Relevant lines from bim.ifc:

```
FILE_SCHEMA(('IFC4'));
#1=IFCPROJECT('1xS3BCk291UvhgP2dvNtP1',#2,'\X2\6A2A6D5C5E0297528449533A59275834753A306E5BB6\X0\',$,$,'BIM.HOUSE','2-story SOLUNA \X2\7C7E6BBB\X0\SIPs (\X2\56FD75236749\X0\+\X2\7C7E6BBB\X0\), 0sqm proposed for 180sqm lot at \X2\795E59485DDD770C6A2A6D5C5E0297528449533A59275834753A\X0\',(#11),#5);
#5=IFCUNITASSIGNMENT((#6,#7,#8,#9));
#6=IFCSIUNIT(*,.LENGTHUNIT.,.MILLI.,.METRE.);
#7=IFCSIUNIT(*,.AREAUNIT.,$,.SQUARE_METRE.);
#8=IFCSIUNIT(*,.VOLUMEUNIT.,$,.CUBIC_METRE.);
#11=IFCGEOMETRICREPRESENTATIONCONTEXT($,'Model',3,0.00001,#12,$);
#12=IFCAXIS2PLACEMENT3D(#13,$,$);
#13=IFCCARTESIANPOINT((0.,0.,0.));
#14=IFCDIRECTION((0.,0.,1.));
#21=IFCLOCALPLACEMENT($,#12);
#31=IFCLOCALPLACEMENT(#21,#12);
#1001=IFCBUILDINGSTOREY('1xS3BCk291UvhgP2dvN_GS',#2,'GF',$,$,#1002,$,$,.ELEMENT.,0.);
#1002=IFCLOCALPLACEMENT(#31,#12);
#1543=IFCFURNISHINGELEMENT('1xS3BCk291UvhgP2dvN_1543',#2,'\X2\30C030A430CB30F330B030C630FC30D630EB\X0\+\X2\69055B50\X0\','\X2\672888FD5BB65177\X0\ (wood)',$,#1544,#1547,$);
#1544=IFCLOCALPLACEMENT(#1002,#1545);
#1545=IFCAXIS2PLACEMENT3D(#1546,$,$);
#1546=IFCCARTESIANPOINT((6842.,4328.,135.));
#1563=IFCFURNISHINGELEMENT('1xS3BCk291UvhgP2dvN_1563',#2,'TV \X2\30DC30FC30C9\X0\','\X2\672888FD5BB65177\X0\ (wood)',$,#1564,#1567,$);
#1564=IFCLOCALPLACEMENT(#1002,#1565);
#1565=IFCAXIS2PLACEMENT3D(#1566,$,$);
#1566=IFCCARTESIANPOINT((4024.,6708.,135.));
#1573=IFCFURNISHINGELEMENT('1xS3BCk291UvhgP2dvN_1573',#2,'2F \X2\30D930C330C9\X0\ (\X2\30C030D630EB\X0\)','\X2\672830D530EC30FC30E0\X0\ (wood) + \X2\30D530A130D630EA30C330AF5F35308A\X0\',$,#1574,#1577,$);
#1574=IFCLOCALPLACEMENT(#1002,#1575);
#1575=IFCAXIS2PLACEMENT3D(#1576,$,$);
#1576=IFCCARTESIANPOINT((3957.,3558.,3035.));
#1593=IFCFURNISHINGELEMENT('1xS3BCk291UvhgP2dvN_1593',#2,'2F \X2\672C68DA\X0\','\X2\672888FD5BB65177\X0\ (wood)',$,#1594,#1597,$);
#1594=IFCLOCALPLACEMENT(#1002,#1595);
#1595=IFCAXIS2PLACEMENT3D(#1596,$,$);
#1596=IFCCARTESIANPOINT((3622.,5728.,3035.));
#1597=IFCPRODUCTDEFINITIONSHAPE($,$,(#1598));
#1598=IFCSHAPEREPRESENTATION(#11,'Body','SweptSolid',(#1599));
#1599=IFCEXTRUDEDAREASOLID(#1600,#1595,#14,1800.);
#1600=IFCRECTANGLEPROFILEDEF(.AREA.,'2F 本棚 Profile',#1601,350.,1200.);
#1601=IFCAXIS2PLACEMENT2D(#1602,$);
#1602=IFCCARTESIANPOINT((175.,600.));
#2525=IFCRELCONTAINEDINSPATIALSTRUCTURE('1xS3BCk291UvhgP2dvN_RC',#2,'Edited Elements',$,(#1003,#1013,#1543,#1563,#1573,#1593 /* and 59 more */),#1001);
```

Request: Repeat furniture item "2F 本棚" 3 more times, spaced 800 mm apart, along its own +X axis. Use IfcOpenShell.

```python
import ifcopenshell
import ifcopenshell.api.geometry
import ifcopenshell.api.root
import ifcopenshell.util.element
import ifcopenshell.util.placement
import ifcopenshell.util.unit

model = ifcopenshell.open("bim.ifc")
unit_scale = ifcopenshell.util.unit.calculate_unit_scale(model)


def reuse_history(source, copy):
    """copy_class also copies each property set's owner history, people and application; keep the originals."""
    for rel in copy.IsDefinedBy:
        if rel.is_a("IfcRelDefinesByProperties") and (history := rel.RelatingPropertyDefinition.OwnerHistory):
            rel.RelatingPropertyDefinition.OwnerHistory = source.OwnerHistory
            ifcopenshell.util.element.remove_deep2(model, history)


source = model.by_guid("1xS3BCk291UvhgP2dvN_1593")
base = ifcopenshell.util.placement.get_local_placement(source.ObjectPlacement)
step = base[:3, 0] * 0.8 / unit_scale

for i in range(1, 4):
    copy = ifcopenshell.api.root.copy_class(model, product=source)
    copy.Representation = ifcopenshell.util.element.copy_deep(
        model, source.Representation, exclude=["IfcGeometricRepresentationContext", "IfcRepresentationMap"]
    )
    reuse_history(source, copy)
    matrix = base.copy()
    matrix[:3, 3] += i * step
    print("added at", matrix[:3, 3].round(3) + 0.0)
    ifcopenshell.api.geometry.edit_object_placement(model, product=copy, matrix=matrix, is_si=False)

model.write("bim_edited.ifc")
```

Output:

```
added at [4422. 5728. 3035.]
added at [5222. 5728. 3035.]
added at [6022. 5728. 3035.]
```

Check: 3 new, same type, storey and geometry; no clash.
